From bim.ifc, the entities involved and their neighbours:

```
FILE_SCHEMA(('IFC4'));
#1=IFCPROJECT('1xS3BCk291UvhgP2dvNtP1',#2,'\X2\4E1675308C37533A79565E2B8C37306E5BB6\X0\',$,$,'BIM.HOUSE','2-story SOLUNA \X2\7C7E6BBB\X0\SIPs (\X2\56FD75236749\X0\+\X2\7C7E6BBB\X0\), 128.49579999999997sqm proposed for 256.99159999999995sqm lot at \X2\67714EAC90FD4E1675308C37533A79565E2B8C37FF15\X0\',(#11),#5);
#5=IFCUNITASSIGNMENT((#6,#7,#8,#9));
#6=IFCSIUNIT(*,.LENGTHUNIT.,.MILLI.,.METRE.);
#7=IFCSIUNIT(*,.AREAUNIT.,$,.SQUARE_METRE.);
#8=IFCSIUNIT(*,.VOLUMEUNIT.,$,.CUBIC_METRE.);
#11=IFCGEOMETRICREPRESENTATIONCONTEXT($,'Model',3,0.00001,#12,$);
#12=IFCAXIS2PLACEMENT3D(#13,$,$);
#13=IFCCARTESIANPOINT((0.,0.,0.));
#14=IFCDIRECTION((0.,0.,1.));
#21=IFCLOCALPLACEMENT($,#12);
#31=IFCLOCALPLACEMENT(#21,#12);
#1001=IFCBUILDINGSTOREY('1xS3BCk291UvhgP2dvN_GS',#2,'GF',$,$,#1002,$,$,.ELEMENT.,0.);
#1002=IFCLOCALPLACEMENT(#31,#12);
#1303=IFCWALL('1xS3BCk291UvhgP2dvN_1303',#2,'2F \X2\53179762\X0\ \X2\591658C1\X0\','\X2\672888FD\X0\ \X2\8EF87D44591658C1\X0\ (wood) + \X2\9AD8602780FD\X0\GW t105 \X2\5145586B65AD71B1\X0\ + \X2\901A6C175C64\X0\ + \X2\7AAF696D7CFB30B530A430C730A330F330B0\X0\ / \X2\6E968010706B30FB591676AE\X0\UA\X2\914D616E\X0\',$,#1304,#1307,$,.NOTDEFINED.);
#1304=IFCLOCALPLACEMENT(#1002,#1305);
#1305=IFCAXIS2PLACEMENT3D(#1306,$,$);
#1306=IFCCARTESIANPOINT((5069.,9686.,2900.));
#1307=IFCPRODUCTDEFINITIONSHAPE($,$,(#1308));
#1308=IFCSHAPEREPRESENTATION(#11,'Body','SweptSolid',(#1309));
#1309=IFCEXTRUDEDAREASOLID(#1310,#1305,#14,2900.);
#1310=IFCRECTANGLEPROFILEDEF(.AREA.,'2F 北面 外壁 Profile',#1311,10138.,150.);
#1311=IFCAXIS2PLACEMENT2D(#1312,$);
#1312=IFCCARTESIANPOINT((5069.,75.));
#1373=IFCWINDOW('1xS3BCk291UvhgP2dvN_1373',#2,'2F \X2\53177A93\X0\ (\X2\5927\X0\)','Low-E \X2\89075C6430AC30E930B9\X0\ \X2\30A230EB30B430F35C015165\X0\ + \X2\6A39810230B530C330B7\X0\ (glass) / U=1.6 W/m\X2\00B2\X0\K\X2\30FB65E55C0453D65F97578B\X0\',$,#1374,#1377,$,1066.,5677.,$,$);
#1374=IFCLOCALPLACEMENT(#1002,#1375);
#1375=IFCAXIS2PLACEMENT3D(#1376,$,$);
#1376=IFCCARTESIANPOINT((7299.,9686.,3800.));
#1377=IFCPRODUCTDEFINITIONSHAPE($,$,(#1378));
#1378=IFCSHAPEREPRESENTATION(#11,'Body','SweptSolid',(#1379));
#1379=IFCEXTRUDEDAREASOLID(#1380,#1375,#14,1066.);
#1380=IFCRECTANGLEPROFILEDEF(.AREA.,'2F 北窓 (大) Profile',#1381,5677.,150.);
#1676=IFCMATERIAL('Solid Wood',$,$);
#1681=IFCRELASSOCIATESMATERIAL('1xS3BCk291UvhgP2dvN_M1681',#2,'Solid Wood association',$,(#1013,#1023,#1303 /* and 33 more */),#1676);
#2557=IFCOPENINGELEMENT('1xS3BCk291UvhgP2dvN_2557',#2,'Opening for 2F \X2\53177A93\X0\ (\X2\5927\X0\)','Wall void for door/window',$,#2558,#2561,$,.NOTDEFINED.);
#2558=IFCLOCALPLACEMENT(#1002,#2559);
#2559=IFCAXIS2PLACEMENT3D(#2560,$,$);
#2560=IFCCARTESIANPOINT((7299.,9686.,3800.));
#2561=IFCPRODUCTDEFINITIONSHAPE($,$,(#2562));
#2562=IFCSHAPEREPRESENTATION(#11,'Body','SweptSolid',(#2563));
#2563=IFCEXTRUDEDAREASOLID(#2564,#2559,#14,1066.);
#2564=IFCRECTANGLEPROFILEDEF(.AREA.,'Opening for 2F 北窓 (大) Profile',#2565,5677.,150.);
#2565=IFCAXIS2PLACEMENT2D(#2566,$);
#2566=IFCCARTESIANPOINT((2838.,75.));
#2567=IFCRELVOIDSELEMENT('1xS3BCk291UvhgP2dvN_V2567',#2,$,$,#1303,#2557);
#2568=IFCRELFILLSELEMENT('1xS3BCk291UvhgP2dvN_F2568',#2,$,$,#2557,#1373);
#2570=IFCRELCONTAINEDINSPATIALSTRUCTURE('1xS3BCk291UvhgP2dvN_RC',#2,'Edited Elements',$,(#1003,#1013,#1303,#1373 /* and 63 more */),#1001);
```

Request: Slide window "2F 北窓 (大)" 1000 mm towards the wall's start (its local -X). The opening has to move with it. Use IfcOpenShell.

```python
import ifcopenshell
import ifcopenshell.api.geometry
import ifcopenshell.util.placement

model = ifcopenshell.open("bim.ifc")

window = model.by_guid("1xS3BCk291UvhgP2dvN_1373")
opening = window.FillsVoids[0].RelatingOpeningElement
wall = opening.VoidsElements[0].RelatingBuildingElement

wall_matrix = ifcopenshell.util.placement.get_local_placement(wall.ObjectPlacement)
shift = wall_matrix[:3, 0] * -1000.0
before = ifcopenshell.util.placement.get_local_placement(window.ObjectPlacement)[:3, 3].copy()

# The window is not placed relative to its opening, so move both.
for product in (opening, window):
    matrix = ifcopenshell.util.placement.get_local_placement(product.ObjectPlacement)
    matrix[:3, 3] += shift
    ifcopenshell.api.geometry.edit_object_placement(model, product=product, matrix=matrix, is_si=False)

after = ifcopenshell.util.placement.get_local_placement(window.ObjectPlacement)[:3, 3]
print("window moved by", (after - before).round(3) + 0.0)

model.write("bim_edited.ifc")
```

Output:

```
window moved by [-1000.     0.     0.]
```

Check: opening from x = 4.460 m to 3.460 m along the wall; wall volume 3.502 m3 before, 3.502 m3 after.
